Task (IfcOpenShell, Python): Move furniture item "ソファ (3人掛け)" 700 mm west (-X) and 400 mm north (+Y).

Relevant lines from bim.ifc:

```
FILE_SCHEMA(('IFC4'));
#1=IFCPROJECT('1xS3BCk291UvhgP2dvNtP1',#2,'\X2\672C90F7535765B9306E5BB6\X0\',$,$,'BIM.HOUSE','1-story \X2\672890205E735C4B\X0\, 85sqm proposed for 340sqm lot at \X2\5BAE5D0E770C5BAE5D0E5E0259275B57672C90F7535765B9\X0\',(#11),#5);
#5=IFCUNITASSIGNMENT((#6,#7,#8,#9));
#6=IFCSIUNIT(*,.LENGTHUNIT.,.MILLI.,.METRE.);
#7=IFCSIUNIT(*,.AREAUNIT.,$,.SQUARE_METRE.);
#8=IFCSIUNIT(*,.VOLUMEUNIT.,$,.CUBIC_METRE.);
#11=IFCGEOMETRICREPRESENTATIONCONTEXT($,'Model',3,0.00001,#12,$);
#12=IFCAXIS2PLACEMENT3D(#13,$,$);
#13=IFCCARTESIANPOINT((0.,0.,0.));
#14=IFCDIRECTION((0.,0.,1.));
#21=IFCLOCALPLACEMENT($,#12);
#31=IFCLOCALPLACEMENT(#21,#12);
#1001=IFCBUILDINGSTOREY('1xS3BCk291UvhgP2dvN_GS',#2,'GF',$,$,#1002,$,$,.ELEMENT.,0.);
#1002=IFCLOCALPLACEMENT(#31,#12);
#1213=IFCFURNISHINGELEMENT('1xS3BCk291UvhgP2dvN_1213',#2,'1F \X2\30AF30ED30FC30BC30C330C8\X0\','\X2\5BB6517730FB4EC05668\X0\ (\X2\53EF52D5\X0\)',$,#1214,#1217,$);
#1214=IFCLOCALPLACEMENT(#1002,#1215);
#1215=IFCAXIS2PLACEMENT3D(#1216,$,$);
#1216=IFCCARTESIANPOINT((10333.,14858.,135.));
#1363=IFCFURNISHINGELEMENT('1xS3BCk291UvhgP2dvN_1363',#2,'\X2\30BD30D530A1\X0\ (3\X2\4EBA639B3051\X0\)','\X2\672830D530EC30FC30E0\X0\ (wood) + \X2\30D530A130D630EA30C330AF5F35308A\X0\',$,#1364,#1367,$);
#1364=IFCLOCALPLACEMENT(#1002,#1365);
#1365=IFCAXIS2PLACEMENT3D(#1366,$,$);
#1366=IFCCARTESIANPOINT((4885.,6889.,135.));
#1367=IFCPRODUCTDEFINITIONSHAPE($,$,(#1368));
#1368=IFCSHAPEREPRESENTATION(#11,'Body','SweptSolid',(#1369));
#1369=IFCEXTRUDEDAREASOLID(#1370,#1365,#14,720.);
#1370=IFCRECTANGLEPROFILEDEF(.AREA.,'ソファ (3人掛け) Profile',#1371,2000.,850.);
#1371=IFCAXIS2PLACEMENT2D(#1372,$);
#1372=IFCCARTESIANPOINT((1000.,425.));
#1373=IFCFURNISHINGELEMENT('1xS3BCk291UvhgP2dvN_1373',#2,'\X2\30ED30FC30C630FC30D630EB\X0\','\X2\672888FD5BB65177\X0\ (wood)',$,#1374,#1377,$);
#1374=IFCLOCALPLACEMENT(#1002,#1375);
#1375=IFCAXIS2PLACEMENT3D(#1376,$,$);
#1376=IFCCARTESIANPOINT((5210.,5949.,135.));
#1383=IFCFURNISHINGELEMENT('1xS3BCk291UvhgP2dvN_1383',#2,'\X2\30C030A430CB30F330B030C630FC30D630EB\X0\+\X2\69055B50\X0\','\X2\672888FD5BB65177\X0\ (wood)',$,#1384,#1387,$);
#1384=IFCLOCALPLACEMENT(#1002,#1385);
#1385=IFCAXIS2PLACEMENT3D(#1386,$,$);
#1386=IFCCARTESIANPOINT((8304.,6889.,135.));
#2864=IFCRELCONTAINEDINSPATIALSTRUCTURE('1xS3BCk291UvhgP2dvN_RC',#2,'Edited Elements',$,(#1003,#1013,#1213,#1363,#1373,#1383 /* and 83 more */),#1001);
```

```python
import ifcopenshell
import ifcopenshell.api.geometry
import ifcopenshell.util.placement
import ifcopenshell.util.unit

model = ifcopenshell.open("bim.ifc")
unit_scale = ifcopenshell.util.unit.calculate_unit_scale(model)

item = model.by_guid("1xS3BCk291UvhgP2dvN_1363")
matrix = ifcopenshell.util.placement.get_local_placement(item.ObjectPlacement)
matrix[0, 3] -= 0.7 / unit_scale
matrix[1, 3] += 0.4 / unit_scale
ifcopenshell.api.geometry.edit_object_placement(model, product=item, matrix=matrix, is_si=False)

print(ifcopenshell.util.placement.get_local_placement(item.ObjectPlacement).round(3) + 0.0)

model.write("bim_updated.ifc")
```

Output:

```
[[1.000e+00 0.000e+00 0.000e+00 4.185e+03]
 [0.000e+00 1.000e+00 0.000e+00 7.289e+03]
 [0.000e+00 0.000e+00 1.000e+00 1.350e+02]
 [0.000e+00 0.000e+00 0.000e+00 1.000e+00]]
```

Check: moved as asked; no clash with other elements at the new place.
